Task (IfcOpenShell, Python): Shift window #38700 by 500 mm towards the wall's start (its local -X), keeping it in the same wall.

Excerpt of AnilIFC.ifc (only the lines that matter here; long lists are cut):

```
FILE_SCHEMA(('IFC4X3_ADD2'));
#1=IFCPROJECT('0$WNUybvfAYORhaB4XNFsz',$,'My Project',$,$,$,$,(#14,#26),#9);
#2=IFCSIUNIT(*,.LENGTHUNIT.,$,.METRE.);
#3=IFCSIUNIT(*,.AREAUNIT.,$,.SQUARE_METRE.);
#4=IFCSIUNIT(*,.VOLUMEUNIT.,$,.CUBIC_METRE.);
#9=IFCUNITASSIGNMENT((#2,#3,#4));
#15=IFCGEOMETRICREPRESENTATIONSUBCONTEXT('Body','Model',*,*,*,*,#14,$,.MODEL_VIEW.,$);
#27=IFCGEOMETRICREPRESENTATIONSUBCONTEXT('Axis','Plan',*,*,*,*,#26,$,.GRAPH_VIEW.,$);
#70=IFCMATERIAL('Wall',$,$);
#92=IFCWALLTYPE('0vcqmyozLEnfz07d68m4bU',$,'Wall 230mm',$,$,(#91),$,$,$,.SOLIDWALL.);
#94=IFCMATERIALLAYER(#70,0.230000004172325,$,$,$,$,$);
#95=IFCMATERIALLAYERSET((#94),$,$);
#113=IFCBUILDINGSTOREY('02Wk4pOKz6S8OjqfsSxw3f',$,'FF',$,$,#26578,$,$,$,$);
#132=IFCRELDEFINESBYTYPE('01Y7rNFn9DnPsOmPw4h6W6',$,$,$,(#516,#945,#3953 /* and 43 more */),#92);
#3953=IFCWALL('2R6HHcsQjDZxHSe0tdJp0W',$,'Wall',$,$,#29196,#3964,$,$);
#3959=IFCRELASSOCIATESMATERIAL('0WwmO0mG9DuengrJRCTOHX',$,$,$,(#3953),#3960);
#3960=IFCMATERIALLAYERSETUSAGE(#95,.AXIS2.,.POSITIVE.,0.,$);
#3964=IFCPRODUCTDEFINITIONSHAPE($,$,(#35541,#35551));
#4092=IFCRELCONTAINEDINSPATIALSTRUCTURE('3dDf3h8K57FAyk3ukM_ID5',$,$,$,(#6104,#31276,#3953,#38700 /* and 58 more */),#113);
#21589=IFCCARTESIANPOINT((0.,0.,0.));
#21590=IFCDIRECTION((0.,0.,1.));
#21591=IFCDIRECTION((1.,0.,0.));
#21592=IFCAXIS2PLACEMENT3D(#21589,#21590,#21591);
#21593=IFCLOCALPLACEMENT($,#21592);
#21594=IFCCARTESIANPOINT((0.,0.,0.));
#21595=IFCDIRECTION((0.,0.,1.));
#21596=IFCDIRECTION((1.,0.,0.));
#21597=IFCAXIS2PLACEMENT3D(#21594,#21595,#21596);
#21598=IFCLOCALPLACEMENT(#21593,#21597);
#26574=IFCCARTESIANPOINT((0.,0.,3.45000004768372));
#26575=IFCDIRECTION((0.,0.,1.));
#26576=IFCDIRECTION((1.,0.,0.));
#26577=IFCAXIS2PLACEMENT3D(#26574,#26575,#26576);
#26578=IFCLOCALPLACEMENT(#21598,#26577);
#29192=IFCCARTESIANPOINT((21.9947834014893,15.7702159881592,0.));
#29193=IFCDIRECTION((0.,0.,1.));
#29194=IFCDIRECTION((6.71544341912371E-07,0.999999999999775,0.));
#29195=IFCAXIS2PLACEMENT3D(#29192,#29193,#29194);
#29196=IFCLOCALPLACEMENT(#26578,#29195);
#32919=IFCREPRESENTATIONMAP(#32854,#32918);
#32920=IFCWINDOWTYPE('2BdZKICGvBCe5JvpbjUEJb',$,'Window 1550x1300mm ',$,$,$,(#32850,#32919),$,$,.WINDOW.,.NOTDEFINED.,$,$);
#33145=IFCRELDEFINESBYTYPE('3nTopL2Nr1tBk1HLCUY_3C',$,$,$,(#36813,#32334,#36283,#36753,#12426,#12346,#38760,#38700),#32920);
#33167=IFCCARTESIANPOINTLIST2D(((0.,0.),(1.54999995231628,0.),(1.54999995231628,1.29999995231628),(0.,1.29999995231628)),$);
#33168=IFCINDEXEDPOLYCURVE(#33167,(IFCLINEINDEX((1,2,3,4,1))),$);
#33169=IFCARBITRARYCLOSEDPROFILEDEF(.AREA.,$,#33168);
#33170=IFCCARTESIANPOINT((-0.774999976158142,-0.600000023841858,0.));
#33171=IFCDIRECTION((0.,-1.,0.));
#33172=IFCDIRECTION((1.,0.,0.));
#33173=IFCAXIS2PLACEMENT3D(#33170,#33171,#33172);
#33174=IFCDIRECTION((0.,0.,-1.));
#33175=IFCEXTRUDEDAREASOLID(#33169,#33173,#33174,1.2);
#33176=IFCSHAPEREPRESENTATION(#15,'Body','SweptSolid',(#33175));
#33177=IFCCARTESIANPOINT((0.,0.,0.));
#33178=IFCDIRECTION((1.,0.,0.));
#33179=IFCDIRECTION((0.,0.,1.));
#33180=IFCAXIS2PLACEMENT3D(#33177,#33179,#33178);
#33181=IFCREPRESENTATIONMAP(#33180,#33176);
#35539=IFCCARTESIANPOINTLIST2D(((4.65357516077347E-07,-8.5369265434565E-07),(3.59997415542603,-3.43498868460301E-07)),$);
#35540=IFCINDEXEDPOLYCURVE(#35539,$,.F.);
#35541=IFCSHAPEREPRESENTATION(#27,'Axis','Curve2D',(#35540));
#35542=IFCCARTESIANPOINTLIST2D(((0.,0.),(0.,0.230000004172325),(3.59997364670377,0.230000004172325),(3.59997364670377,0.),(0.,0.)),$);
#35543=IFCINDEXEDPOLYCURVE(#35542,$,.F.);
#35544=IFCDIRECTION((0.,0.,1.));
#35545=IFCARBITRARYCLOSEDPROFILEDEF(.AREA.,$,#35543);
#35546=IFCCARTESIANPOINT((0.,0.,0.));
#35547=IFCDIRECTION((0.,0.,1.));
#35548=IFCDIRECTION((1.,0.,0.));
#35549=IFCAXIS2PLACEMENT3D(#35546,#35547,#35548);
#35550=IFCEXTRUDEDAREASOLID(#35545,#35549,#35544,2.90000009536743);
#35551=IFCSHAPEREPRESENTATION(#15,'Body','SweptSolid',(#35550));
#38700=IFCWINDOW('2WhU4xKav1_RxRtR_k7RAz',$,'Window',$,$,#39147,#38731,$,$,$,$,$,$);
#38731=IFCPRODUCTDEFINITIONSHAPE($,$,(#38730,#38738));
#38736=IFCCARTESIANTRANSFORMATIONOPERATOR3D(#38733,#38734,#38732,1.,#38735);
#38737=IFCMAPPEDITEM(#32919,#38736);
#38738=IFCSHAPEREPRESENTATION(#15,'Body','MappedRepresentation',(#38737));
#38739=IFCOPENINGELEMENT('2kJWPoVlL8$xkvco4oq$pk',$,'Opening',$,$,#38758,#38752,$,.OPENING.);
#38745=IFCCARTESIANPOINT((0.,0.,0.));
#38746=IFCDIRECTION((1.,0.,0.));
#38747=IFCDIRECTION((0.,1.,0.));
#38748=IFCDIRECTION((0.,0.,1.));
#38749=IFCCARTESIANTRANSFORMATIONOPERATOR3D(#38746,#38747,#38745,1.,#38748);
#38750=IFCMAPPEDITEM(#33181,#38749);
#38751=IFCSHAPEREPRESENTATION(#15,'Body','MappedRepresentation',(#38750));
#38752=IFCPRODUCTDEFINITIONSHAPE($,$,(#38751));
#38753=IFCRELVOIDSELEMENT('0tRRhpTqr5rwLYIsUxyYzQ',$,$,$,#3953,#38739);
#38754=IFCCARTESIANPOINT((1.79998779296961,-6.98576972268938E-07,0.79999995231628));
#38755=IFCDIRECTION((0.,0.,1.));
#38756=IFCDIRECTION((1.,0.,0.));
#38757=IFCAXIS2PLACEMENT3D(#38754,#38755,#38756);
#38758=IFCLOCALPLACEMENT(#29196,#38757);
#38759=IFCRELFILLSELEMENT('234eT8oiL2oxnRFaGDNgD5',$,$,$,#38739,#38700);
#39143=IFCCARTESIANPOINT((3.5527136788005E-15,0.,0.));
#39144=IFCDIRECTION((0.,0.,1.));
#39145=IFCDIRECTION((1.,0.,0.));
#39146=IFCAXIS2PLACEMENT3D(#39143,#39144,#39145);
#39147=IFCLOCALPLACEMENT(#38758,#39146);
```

```python
import ifcopenshell
import ifcopenshell.api.geometry
import ifcopenshell.util.placement
import ifcopenshell.util.unit

model = ifcopenshell.open("AnilIFC.ifc")
unit_scale = ifcopenshell.util.unit.calculate_unit_scale(model)

window = model.by_guid("2WhU4xKav1_RxRtR_k7RAz")
opening = window.FillsVoids[0].RelatingOpeningElement
wall = opening.VoidsElements[0].RelatingBuildingElement

wall_matrix = ifcopenshell.util.placement.get_local_placement(wall.ObjectPlacement)
shift = wall_matrix[:3, 0] * -0.5 / unit_scale
before = ifcopenshell.util.placement.get_local_placement(window.ObjectPlacement)[:3, 3].copy()

# The window is placed relative to its opening, so it follows when the opening moves.
matrix = ifcopenshell.util.placement.get_local_placement(opening.ObjectPlacement)
matrix[:3, 3] += shift
ifcopenshell.api.geometry.edit_object_placement(
    model, product=opening, matrix=matrix, is_si=False, should_transform_children=True
)

after = ifcopenshell.util.placement.get_local_placement(window.ObjectPlacement)[:3, 3]
print("window moved by", (after - before).round(3) + 0.0)

model.write("AnilIFC_edited.ifc")
```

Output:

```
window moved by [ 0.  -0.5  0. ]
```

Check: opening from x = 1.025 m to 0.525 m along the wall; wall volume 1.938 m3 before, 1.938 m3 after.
